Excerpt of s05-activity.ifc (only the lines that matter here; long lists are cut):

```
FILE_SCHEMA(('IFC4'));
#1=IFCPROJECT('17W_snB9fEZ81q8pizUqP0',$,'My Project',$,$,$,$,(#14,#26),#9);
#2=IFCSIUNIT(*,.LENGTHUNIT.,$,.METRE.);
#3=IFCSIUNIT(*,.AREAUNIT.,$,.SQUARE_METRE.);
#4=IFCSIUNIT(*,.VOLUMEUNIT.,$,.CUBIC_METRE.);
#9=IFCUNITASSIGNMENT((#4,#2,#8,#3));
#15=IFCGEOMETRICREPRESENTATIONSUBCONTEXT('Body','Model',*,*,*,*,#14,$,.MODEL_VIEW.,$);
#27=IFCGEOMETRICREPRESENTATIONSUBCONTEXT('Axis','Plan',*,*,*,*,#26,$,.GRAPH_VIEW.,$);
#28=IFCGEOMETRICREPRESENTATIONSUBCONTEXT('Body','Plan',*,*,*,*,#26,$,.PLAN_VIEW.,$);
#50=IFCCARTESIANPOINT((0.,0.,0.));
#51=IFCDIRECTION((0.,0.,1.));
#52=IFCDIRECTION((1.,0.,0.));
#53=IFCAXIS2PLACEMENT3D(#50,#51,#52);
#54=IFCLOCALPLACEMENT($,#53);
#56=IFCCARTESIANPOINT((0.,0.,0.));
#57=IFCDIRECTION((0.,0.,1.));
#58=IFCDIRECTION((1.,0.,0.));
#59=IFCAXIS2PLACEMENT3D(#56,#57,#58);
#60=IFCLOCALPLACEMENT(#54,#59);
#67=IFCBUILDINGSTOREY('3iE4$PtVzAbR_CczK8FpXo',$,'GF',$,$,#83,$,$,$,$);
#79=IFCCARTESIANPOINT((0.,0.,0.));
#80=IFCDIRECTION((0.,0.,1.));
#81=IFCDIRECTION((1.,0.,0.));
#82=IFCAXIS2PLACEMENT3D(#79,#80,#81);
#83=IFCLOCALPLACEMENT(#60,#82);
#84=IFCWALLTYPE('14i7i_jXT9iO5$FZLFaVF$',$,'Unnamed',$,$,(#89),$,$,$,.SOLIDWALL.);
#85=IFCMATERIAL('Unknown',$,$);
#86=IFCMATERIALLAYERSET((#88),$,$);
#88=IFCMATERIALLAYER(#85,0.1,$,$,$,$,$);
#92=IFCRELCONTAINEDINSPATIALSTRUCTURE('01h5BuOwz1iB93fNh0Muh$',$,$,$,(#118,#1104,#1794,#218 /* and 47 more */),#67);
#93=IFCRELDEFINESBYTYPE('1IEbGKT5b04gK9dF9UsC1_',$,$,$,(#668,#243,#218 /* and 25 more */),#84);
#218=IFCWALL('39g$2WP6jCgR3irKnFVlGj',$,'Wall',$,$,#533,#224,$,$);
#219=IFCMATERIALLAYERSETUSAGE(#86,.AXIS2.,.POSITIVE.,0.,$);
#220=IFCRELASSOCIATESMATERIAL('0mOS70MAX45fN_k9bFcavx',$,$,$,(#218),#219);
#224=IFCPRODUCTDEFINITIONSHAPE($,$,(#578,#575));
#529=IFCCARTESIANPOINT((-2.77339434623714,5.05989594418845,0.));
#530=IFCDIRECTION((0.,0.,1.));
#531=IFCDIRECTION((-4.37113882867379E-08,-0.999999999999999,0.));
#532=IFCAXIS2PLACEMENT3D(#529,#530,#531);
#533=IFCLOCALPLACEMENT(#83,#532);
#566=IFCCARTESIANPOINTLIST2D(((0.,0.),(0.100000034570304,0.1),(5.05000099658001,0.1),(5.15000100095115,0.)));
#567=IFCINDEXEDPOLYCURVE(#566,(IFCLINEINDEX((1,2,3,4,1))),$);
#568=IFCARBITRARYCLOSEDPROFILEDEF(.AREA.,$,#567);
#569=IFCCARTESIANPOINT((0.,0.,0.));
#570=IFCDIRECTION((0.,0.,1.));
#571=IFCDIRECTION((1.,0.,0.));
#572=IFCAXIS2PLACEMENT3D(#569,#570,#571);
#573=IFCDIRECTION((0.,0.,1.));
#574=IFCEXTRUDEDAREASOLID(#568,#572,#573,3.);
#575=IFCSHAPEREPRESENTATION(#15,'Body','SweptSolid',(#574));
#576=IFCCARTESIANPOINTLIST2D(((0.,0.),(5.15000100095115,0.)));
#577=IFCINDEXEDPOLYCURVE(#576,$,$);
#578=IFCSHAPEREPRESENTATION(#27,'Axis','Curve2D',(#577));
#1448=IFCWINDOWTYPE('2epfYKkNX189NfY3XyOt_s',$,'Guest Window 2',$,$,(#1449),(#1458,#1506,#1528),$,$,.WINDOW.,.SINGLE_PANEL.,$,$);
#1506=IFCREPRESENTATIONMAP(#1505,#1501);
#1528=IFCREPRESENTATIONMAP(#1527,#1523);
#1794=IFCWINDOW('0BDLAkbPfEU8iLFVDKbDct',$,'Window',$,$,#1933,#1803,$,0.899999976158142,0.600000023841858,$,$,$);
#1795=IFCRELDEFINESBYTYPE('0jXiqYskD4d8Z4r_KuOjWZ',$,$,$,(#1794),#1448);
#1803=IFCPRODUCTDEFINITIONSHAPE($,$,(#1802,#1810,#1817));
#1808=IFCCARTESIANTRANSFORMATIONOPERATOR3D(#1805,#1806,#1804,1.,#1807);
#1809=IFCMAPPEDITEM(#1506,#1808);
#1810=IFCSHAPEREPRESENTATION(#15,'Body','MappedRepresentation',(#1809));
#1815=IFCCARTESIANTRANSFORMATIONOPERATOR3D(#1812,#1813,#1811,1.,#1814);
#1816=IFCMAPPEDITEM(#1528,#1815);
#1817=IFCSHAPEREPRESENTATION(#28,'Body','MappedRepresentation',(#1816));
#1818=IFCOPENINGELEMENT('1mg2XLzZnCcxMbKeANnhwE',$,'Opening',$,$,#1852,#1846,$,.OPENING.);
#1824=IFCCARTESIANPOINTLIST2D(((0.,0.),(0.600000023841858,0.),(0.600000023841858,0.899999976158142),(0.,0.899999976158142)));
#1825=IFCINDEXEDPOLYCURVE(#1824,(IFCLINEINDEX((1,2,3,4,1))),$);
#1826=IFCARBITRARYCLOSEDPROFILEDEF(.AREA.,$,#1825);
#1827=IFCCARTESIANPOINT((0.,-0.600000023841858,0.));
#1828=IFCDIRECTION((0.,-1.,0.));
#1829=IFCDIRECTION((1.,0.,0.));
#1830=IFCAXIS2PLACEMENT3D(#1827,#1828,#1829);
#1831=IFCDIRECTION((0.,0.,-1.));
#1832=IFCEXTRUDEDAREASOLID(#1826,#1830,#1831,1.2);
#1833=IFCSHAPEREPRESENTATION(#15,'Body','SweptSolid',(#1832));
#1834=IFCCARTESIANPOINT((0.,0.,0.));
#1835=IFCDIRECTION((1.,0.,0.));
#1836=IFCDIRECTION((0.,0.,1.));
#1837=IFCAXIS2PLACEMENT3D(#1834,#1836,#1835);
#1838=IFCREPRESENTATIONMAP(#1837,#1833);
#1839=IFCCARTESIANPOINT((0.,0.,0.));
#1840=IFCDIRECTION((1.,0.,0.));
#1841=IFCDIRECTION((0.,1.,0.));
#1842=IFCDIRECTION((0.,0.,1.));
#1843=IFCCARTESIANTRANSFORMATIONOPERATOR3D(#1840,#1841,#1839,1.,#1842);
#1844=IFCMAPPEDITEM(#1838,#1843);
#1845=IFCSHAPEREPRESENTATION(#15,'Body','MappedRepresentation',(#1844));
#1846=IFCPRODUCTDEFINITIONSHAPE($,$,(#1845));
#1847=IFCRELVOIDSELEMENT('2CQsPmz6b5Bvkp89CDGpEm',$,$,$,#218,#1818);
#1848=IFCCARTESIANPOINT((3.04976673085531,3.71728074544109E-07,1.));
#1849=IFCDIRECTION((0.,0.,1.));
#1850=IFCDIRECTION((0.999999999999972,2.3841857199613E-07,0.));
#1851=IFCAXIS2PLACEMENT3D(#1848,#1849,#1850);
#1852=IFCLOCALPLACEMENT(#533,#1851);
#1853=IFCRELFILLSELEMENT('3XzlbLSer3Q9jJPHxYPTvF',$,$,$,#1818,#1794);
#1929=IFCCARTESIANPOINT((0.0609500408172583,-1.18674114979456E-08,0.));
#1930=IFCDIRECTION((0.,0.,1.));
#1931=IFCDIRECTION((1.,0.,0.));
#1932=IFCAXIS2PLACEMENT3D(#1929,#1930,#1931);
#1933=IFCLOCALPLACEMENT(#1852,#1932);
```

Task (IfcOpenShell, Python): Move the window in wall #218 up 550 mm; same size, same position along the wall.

```python
import numpy as np
import ifcopenshell
import ifcopenshell.api.geometry
import ifcopenshell.util.placement
import ifcopenshell.util.unit

model = ifcopenshell.open("s05-activity.ifc")
unit_scale = ifcopenshell.util.unit.calculate_unit_scale(model)

window = model.by_guid("0BDLAkbPfEU8iLFVDKbDct")
opening = window.FillsVoids[0].RelatingOpeningElement
dz = 0.55 / unit_scale

shift = np.array([0.0, 0.0, dz])
# The window is placed relative to its opening, so it follows when the opening moves.
matrix = ifcopenshell.util.placement.get_local_placement(opening.ObjectPlacement)
matrix[:3, 3] += shift
ifcopenshell.api.geometry.edit_object_placement(
    model, product=opening, matrix=matrix, is_si=False, should_transform_children=True
)

print(f"moved by {dz * unit_scale:+.3f} m")

model.write("s05-activity_updated.ifc")
```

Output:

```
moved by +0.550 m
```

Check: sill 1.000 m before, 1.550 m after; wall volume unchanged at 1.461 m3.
